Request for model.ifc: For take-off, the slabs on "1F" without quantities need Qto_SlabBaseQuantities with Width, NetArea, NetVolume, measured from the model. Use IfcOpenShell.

First a look at what the model holds.

```python
import ifcopenshell
import ifcopenshell.util.element
import ifcopenshell.util.unit

model = ifcopenshell.open("model.ifc")
print(model.schema)
for unit_type in ("LENGTHUNIT", "AREAUNIT", "VOLUMEUNIT"):
    print(unit_type, ifcopenshell.util.unit.calculate_unit_scale(model, unit_type))
storey = next(s for s in model.by_type("IfcBuildingStorey") if s.Name == "1F")
slabs = [e for e in ifcopenshell.util.element.get_decomposition(storey) if e.is_a("IfcSlab")]
for e in sorted(slabs, key=lambda e: e.id()):
    print(e.id(), e.is_a(), e.Name, list(ifcopenshell.util.element.get_psets(e, qtos_only=True)), sep=" | ")
```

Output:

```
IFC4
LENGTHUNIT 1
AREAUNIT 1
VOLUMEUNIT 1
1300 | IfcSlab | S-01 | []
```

```python
import ifcopenshell
import ifcopenshell.api.pset
import ifcopenshell.geom
import ifcopenshell.util.element
import ifcopenshell.util.shape
import ifcopenshell.util.unit

model = ifcopenshell.open("model.ifc")
unit_scale = ifcopenshell.util.unit.calculate_unit_scale(model)
area_scale = ifcopenshell.util.unit.calculate_unit_scale(model, "AREAUNIT")
volume_scale = ifcopenshell.util.unit.calculate_unit_scale(model, "VOLUMEUNIT")
settings = ifcopenshell.geom.settings()

storey = next(s for s in model.by_type("IfcBuildingStorey") if s.Name == "1F")
slabs = [e for e in ifcopenshell.util.element.get_decomposition(storey) if e.is_a("IfcSlab")]

for e in sorted(slabs, key=lambda e: e.id()):
    if ifcopenshell.util.element.get_psets(e, qtos_only=True, should_inherit=False):
        continue
    # Geometry comes back in metres, in the element's own axes.
    shape = ifcopenshell.geom.create_shape(settings, e)
    values = {
        "Width": ifcopenshell.util.shape.get_z(shape.geometry) / unit_scale,
        "NetArea": ifcopenshell.util.shape.get_footprint_area(shape.geometry) / area_scale,
        "NetVolume": ifcopenshell.util.shape.get_volume(shape.geometry) / volume_scale,
    }
    qto = ifcopenshell.api.pset.add_qto(model, product=e, name="Qto_SlabBaseQuantities")
    ifcopenshell.api.pset.edit_qto(model, qto=qto, properties=values)
    print(e.id(), {k: round(v, 3) for k, v in values.items()})

model.write("model_v2.ifc")
```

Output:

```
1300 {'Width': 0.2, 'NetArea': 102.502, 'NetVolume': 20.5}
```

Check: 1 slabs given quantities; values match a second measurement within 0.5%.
